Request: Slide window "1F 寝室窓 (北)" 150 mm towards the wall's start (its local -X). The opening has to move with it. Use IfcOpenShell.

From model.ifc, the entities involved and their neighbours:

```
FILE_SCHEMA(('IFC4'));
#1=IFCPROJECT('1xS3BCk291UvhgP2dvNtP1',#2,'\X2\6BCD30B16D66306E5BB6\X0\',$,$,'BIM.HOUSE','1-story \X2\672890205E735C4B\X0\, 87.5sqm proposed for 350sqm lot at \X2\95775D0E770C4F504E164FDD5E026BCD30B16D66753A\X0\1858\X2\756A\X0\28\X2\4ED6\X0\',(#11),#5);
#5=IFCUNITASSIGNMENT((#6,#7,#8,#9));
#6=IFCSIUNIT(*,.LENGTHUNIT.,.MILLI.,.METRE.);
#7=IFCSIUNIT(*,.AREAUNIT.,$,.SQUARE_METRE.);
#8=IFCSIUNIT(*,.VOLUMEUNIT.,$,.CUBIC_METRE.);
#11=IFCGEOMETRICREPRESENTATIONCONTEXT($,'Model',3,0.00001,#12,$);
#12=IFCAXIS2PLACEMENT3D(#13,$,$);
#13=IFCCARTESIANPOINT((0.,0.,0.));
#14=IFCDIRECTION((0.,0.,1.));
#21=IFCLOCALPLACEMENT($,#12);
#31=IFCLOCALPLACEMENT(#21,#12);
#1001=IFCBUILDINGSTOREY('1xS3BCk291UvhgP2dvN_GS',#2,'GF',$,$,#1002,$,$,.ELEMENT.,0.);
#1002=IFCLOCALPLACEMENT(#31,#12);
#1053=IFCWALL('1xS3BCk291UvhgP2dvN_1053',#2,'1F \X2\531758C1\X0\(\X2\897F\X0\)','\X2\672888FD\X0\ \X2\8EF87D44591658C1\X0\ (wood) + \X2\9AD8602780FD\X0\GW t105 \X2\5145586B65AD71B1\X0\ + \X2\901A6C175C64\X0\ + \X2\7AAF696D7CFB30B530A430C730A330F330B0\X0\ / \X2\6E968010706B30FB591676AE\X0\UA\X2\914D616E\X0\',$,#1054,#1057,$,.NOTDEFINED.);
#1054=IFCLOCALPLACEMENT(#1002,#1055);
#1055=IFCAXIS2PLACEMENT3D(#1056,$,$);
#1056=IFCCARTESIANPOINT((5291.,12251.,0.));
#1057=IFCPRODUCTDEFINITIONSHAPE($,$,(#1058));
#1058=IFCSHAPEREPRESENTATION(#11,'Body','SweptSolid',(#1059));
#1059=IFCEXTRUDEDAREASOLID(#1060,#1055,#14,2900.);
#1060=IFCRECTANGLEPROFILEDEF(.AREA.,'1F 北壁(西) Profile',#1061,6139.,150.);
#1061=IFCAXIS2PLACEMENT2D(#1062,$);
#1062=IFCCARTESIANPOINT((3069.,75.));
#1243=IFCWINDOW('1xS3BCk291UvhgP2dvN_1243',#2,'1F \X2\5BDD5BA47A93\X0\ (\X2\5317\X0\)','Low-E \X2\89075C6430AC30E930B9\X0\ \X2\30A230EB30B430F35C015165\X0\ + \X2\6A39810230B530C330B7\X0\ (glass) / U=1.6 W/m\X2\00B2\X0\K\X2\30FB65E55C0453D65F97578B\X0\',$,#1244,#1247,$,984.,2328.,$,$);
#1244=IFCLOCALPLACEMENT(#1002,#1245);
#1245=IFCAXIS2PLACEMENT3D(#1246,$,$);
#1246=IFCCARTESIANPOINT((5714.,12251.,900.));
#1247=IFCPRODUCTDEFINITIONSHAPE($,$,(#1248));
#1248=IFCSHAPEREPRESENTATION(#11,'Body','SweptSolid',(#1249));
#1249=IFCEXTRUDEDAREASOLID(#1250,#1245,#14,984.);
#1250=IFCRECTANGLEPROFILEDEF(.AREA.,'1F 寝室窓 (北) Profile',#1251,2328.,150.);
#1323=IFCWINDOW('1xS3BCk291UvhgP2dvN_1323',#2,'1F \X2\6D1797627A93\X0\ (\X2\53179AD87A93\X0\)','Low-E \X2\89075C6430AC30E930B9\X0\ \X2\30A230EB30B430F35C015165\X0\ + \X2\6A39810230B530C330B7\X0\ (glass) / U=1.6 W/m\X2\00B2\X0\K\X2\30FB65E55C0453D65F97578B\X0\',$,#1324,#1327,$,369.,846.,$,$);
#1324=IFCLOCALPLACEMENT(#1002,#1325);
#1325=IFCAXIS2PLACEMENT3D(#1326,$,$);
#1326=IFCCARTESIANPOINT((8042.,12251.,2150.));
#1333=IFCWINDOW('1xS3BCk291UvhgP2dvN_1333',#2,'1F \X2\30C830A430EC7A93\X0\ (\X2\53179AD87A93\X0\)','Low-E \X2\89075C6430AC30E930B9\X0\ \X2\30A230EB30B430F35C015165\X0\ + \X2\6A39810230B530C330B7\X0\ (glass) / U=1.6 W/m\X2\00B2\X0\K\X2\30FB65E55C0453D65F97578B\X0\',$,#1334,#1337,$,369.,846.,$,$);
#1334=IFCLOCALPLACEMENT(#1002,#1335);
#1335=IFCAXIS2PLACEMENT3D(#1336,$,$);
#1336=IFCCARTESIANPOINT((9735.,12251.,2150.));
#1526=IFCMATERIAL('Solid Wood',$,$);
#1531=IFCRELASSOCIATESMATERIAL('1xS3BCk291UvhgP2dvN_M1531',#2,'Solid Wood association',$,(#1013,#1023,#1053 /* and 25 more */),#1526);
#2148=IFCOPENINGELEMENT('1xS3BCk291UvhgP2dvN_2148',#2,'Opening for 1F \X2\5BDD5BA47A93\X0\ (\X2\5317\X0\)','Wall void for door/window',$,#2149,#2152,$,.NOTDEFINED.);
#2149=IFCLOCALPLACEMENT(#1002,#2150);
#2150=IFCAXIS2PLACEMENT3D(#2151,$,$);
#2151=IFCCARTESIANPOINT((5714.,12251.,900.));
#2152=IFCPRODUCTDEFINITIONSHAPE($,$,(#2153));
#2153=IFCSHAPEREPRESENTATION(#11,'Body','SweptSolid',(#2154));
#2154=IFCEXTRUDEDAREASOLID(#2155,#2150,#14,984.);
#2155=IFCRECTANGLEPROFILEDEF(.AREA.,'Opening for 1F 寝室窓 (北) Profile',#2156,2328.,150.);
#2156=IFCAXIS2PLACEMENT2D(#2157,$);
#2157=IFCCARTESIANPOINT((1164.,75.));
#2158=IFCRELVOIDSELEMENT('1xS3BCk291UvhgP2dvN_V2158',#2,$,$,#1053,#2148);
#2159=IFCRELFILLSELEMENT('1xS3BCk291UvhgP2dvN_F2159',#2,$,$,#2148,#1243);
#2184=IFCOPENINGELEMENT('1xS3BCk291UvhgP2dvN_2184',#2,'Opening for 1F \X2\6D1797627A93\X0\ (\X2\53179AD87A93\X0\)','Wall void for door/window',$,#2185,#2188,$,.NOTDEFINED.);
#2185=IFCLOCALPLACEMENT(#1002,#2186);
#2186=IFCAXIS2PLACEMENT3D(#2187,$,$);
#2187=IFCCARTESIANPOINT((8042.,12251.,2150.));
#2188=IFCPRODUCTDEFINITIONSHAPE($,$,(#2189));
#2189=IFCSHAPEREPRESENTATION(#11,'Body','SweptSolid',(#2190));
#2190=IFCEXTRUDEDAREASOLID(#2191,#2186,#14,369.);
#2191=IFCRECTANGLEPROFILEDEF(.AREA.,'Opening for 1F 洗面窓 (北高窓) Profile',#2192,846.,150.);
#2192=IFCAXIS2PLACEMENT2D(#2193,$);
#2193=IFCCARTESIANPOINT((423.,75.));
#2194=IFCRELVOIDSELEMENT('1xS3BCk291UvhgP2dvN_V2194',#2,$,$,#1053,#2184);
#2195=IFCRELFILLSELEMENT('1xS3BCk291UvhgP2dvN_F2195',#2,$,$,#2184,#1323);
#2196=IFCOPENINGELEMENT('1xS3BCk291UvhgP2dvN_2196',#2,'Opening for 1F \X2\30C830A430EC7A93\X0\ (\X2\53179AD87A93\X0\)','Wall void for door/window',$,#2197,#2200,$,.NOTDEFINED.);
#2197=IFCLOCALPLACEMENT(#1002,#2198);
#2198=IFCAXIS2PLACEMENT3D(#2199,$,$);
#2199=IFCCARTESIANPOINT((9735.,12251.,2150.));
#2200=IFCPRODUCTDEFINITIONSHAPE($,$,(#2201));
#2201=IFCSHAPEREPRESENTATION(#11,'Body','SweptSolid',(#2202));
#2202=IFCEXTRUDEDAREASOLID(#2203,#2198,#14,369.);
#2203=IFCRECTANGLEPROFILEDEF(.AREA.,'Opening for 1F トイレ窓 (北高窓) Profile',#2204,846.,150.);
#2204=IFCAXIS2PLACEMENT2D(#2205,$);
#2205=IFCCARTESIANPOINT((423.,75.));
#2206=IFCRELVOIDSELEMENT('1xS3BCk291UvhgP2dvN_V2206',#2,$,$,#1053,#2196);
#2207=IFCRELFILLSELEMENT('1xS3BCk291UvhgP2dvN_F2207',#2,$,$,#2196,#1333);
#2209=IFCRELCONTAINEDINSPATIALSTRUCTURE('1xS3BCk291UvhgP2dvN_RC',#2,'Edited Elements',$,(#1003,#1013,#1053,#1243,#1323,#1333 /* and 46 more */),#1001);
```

```python
import ifcopenshell
import ifcopenshell.api.geometry
import ifcopenshell.util.placement
import ifcopenshell.util.unit

model = ifcopenshell.open("model.ifc")
unit_scale = ifcopenshell.util.unit.calculate_unit_scale(model)

window = model.by_guid("1xS3BCk291UvhgP2dvN_1243")
opening = window.FillsVoids[0].RelatingOpeningElement
wall = opening.VoidsElements[0].RelatingBuildingElement

wall_matrix = ifcopenshell.util.placement.get_local_placement(wall.ObjectPlacement)
shift = wall_matrix[:3, 0] * -0.15 / unit_scale
before = ifcopenshell.util.placement.get_local_placement(window.ObjectPlacement)[:3, 3].copy()

# The window is not placed relative to its opening, so move both.
for product in (opening, window):
    matrix = ifcopenshell.util.placement.get_local_placement(product.ObjectPlacement)
    matrix[:3, 3] += shift
    ifcopenshell.api.geometry.edit_object_placement(model, product=product, matrix=matrix, is_si=False)

after = ifcopenshell.util.placement.get_local_placement(window.ObjectPlacement)[:3, 3]
print("window moved by", (after - before).round(3) + 0.0)

model.write("model-out.ifc")
```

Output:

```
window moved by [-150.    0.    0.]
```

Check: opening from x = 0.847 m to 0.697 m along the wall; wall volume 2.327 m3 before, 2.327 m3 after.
